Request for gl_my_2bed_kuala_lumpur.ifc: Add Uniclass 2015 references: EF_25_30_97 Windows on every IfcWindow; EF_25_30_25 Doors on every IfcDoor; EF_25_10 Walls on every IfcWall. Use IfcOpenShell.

First a look at what the model holds.

```python
import ifcopenshell

model = ifcopenshell.open("gl_my_2bed_kuala_lumpur.ifc")
print(model.schema)
print("classifications:", [c.Name for c in model.by_type("IfcClassification")])
for ifc_class in ("IfcDoor", "IfcRoof", "IfcStair", "IfcWall", "IfcWindow"):
    print(ifc_class, len(model.by_type(ifc_class)))
```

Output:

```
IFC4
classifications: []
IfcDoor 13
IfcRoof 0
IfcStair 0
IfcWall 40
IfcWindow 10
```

```python
import ifcopenshell
import ifcopenshell.api.classification

model = ifcopenshell.open("gl_my_2bed_kuala_lumpur.ifc")

system = ifcopenshell.api.classification.add_classification(model, classification="Uniclass 2015")

codes = {
    "IfcWindow": ("EF_25_30_97", "Windows"),
    "IfcDoor": ("EF_25_30_25", "Doors"),
    "IfcWall": ("EF_25_10", "Walls"),
}
for ifc_class, (code, name) in codes.items():
    products = model.by_type(ifc_class)
    ifcopenshell.api.classification.add_reference(
        model, products=products, classification=system, identification=code, name=name
    )
    print(code, len(products))

model.write("gl_my_2bed_kuala_lumpur_rev.ifc")
```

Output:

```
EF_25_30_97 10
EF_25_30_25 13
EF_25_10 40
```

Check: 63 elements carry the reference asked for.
